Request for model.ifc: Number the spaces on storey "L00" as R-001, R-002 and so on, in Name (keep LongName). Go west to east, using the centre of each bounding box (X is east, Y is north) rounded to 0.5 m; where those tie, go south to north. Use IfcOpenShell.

First a look at what the model holds.

```python
import ifcopenshell
import ifcopenshell.util.element
import ifcopenshell.util.placement

model = ifcopenshell.open("model.ifc")
print(model.schema)
storey = next(s for s in model.by_type("IfcBuildingStorey") if s.Name == "L00")
spaces = [e for e in ifcopenshell.util.element.get_decomposition(storey) if e.is_a("IfcSpace")]
for e in sorted(spaces, key=lambda e: e.id()):
    origin = ifcopenshell.util.placement.get_local_placement(e.ObjectPlacement)[:3, 3]
    print(e.id(), e.Name, e.LongName, origin.round(2) + 0.0, sep=" | ")
```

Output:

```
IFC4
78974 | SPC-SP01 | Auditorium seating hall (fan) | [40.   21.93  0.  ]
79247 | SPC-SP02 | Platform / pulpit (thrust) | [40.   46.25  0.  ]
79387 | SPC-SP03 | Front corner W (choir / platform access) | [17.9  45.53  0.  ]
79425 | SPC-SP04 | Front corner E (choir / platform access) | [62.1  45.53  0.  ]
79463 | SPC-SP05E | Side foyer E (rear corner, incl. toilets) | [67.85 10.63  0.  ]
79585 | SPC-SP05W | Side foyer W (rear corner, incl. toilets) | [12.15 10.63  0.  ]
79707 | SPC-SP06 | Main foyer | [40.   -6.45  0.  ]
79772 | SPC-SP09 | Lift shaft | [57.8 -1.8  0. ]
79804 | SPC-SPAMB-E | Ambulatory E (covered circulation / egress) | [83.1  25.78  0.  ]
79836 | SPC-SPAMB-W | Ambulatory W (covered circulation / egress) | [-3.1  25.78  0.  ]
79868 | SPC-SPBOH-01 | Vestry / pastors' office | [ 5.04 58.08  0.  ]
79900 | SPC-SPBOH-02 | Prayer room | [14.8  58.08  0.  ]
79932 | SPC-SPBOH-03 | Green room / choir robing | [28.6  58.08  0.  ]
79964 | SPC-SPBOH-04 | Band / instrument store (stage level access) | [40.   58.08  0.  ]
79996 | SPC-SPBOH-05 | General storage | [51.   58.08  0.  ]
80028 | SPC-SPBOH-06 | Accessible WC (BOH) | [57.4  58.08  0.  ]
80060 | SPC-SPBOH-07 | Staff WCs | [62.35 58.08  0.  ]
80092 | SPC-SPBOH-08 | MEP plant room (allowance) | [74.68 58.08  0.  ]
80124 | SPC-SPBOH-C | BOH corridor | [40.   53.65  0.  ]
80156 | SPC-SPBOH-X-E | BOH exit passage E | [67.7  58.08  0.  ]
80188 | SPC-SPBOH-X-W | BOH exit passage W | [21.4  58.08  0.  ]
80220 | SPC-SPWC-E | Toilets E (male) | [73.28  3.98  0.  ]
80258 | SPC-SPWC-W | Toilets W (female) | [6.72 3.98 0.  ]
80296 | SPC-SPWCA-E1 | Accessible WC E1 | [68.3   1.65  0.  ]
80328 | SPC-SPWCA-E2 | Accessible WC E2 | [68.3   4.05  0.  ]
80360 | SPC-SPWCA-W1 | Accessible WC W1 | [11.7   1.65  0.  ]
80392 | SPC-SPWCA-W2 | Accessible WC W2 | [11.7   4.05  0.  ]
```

```python
import ifcopenshell
import ifcopenshell.geom
import ifcopenshell.util.element
import ifcopenshell.util.shape

model = ifcopenshell.open("model.ifc")
settings = ifcopenshell.geom.settings()
settings.set("use-world-coords", True)


def centre(element):
    shape = ifcopenshell.geom.create_shape(settings, element)
    return ifcopenshell.util.shape.get_bbox_centroid(shape.geometry)


storey = next(s for s in model.by_type("IfcBuildingStorey") if s.Name == "L00")
spaces = [e for e in ifcopenshell.util.element.get_decomposition(storey) if e.is_a("IfcSpace")]

# Insertion points can sit at a corner or the storey origin, so sort by the geometry (in metres).
centres = {e: centre(e) for e in spaces}
spaces.sort(key=lambda e: (round(centres[e][0] / 0.5), centres[e][1]))

for i, e in enumerate(spaces, start=1):
    number = f"R-0{i:02d}"
    e.Name = number
    print(e.id(), number)

model.write("model_updated.ifc")
```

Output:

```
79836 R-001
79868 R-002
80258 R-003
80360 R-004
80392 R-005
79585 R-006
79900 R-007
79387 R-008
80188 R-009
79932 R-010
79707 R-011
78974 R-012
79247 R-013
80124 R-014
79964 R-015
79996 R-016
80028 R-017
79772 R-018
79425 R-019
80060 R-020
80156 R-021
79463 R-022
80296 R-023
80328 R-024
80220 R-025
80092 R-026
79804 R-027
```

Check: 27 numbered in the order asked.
